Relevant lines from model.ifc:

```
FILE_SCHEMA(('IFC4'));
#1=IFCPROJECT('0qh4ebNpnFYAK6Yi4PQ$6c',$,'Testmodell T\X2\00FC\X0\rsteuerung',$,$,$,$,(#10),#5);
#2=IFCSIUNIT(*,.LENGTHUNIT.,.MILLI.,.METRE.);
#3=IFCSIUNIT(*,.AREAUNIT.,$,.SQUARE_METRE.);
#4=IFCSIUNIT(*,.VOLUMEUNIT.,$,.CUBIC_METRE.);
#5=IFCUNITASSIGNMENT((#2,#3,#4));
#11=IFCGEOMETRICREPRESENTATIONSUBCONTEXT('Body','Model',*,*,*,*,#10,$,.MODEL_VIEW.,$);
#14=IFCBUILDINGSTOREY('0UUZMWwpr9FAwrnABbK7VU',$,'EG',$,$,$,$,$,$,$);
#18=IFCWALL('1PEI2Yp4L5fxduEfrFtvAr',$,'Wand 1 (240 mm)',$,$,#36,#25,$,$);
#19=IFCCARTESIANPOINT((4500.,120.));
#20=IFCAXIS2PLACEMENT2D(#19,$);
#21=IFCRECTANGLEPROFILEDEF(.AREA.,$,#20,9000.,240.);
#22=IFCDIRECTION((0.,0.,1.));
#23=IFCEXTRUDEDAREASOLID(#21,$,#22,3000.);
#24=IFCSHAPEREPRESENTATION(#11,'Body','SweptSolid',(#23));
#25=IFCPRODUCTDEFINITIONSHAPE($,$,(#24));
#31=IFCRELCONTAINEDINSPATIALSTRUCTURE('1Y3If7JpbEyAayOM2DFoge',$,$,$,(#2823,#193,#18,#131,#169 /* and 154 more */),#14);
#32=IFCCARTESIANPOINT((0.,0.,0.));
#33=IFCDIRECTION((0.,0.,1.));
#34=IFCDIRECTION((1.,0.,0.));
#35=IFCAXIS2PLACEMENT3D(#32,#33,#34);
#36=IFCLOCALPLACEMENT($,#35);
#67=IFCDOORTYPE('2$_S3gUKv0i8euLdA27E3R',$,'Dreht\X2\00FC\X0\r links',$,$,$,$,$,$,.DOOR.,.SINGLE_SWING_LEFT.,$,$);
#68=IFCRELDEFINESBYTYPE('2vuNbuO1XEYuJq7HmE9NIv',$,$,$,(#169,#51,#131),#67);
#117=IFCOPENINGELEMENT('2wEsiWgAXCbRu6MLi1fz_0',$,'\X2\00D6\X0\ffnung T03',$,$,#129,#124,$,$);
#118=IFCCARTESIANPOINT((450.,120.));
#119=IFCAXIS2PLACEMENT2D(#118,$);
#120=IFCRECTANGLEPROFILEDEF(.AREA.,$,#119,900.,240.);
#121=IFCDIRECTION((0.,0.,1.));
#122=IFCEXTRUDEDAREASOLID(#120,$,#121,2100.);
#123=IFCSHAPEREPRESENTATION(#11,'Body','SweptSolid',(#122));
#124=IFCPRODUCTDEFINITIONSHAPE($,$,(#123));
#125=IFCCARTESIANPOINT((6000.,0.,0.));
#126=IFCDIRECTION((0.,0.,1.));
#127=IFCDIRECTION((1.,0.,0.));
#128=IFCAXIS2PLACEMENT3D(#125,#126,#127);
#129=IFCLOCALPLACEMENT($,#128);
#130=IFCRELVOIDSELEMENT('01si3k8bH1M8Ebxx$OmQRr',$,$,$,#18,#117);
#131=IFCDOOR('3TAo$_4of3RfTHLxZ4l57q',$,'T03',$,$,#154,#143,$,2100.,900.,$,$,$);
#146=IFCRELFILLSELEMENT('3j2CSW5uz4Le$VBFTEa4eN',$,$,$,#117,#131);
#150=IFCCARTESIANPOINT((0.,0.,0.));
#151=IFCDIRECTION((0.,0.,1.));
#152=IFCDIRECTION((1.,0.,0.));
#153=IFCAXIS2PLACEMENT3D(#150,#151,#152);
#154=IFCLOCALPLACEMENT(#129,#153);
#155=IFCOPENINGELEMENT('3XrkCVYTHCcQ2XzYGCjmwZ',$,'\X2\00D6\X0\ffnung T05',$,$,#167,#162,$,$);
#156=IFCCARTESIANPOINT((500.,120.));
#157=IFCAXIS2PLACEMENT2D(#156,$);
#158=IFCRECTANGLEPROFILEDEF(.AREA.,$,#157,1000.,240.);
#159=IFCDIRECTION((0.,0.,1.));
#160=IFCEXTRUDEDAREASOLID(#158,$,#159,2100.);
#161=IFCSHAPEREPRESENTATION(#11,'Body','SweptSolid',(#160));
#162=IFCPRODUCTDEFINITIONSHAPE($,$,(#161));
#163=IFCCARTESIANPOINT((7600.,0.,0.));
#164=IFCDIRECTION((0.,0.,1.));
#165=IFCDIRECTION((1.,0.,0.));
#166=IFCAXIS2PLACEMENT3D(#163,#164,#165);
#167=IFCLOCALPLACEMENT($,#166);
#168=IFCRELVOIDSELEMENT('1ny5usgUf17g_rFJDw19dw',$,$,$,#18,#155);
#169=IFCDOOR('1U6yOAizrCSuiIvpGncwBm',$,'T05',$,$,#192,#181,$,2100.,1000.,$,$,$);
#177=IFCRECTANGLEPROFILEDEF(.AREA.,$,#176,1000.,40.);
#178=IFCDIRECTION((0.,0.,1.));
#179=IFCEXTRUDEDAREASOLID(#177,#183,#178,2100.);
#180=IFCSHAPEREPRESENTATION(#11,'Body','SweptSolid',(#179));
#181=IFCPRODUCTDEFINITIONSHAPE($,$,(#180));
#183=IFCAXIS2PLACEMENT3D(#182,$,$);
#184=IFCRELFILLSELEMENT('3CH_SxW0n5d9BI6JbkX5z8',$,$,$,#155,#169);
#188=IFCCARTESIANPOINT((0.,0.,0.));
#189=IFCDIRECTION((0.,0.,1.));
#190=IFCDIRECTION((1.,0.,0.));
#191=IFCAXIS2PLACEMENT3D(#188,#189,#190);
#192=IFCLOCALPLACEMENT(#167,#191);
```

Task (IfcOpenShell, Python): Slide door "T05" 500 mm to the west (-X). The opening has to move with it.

```python
import ifcopenshell
import ifcopenshell.api.geometry
import ifcopenshell.util.placement
import ifcopenshell.util.unit

model = ifcopenshell.open("model.ifc")
unit_scale = ifcopenshell.util.unit.calculate_unit_scale(model)

door = model.by_id(169)
opening = door.FillsVoids[0].RelatingOpeningElement
wall = opening.VoidsElements[0].RelatingBuildingElement

wall_matrix = ifcopenshell.util.placement.get_local_placement(wall.ObjectPlacement)
shift = wall_matrix[:3, 0] * -0.5 / unit_scale
before = ifcopenshell.util.placement.get_local_placement(door.ObjectPlacement)[:3, 3].copy()

# The door is placed relative to its opening, so it follows when the opening moves.
matrix = ifcopenshell.util.placement.get_local_placement(opening.ObjectPlacement)
matrix[:3, 3] += shift
ifcopenshell.api.geometry.edit_object_placement(
    model, product=opening, matrix=matrix, is_si=False, should_transform_children=True
)

after = ifcopenshell.util.placement.get_local_placement(door.ObjectPlacement)[:3, 3]
print("door moved by", (after - before).round(3) + 0.0)

model.write("model_rev.ifc")
```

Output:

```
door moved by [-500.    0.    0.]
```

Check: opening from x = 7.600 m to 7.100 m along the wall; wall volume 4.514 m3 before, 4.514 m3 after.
